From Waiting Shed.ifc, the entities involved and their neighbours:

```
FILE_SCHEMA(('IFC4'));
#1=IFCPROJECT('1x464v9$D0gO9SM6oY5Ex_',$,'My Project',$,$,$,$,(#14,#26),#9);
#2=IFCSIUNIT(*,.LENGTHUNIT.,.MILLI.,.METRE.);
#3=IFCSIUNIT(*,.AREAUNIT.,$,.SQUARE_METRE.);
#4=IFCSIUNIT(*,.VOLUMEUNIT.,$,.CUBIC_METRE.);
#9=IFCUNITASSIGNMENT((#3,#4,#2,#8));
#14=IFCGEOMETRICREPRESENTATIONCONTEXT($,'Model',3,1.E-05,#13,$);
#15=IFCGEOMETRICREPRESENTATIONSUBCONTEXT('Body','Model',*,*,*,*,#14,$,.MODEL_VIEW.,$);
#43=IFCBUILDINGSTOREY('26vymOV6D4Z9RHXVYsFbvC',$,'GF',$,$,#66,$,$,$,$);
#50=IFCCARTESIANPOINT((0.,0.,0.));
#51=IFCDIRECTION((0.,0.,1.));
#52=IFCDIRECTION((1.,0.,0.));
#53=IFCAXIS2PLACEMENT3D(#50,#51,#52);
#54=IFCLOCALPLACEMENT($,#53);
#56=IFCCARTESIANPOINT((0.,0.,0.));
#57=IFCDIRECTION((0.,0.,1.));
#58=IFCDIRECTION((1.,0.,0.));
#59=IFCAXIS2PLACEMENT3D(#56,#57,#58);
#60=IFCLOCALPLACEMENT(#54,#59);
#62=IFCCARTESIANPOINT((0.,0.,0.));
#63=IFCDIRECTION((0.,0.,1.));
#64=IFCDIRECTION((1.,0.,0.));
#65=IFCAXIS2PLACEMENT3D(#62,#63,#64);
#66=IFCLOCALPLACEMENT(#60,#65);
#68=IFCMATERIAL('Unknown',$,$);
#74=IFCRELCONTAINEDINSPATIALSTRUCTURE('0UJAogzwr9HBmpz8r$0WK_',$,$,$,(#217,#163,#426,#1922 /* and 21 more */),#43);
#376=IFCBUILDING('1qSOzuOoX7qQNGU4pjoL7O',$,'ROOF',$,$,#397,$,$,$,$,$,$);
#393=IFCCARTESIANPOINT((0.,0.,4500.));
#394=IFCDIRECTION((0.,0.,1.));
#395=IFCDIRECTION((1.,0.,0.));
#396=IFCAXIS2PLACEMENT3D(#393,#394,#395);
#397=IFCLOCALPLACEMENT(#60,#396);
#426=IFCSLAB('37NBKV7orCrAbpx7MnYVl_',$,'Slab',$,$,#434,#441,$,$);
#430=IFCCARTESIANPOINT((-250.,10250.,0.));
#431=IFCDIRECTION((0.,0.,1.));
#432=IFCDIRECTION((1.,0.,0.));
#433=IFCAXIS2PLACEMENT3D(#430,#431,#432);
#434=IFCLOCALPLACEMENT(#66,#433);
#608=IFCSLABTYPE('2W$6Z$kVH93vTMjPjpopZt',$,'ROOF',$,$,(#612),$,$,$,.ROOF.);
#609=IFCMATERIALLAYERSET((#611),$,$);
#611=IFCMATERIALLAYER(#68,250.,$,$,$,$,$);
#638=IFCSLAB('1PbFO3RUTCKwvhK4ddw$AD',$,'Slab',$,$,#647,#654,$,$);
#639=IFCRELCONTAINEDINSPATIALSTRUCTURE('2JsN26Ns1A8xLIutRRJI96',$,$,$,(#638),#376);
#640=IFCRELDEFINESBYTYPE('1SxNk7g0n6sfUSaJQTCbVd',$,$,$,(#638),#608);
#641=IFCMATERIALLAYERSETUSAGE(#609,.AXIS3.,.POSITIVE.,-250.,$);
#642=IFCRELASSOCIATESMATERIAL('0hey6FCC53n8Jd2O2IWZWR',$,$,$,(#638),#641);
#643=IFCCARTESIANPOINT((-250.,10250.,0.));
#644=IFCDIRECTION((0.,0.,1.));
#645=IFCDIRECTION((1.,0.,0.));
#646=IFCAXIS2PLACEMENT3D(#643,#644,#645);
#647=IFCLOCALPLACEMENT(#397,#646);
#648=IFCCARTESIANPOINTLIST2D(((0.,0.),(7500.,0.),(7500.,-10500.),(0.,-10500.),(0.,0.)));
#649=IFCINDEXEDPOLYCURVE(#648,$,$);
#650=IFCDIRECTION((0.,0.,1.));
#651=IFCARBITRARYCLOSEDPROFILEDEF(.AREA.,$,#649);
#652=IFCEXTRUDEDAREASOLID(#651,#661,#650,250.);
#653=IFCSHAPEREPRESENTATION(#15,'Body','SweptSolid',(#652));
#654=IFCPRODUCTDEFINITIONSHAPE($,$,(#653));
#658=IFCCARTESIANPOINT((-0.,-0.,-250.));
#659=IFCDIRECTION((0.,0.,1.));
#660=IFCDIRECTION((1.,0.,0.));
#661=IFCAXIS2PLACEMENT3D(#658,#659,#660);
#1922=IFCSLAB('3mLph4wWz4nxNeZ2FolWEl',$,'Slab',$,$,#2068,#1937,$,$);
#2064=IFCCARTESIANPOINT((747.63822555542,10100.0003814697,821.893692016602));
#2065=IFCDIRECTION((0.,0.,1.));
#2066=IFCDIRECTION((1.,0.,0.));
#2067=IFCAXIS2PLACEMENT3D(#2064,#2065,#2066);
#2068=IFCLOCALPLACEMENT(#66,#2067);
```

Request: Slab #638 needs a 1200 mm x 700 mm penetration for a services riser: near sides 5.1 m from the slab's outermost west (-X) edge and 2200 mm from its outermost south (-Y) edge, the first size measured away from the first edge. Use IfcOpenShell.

```python
import numpy as np
import ifcopenshell
import ifcopenshell.api.feature
import ifcopenshell.api.geometry
import ifcopenshell.api.root
import ifcopenshell.geom
import ifcopenshell.util.placement
import ifcopenshell.util.representation
import ifcopenshell.util.shape
import ifcopenshell.util.unit

model = ifcopenshell.open("Waiting Shed.ifc")
unit_scale = ifcopenshell.util.unit.calculate_unit_scale(model)
settings = ifcopenshell.geom.settings()


def volume(element):
    """Net volume in cubic metres, openings subtracted."""
    shape = ifcopenshell.geom.create_shape(settings, element)
    return ifcopenshell.util.shape.get_volume(shape.geometry)


slab = model.by_id(638)
before = volume(slab)

# Extent in the slab's own axes, in metres. The edges named are its -X and -Y sides.
slab_shape = ifcopenshell.geom.create_shape(settings, slab)
vertices = ifcopenshell.util.shape.get_vertices(slab_shape.geometry)
x_min, y_min, bottom = vertices.min(axis=0)
top = vertices[:, 2].max()

opening = ifcopenshell.api.root.create_entity(model, ifc_class="IfcOpeningElement", name="Services riser opening", predefined_type="OPENING")
context = ifcopenshell.util.representation.get_context(model, "Model", "Body", "MODEL_VIEW")
width, depth = 1.2, 0.7
outline = [(0.0, 0.0), (width, 0.0), (width, depth), (0.0, depth), (0.0, 0.0)]
# Overshoot both faces by 50 mm so the cut is clean.
shape = ifcopenshell.api.geometry.add_slab_representation(
    model, context=context, depth=top - bottom + 0.1, polyline=outline
)
ifcopenshell.api.geometry.assign_representation(model, product=opening, representation=shape)

matrix = ifcopenshell.util.placement.get_local_placement(slab.ObjectPlacement)
matrix[:, 3] = matrix @ np.append(np.array([x_min + 5.1, y_min + 2.2, bottom - 0.05]) / unit_scale, 1.0)
ifcopenshell.api.geometry.edit_object_placement(model, product=opening, matrix=matrix, is_si=False)
ifcopenshell.api.feature.add_feature(model, feature=opening, element=slab)

after = volume(slab)

print(f"slab volume {before:.3f} -> {after:.3f} m3")

model.write("Waiting Shed_v2.ifc")
```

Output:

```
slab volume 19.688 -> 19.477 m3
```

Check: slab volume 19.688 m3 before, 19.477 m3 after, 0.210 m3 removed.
